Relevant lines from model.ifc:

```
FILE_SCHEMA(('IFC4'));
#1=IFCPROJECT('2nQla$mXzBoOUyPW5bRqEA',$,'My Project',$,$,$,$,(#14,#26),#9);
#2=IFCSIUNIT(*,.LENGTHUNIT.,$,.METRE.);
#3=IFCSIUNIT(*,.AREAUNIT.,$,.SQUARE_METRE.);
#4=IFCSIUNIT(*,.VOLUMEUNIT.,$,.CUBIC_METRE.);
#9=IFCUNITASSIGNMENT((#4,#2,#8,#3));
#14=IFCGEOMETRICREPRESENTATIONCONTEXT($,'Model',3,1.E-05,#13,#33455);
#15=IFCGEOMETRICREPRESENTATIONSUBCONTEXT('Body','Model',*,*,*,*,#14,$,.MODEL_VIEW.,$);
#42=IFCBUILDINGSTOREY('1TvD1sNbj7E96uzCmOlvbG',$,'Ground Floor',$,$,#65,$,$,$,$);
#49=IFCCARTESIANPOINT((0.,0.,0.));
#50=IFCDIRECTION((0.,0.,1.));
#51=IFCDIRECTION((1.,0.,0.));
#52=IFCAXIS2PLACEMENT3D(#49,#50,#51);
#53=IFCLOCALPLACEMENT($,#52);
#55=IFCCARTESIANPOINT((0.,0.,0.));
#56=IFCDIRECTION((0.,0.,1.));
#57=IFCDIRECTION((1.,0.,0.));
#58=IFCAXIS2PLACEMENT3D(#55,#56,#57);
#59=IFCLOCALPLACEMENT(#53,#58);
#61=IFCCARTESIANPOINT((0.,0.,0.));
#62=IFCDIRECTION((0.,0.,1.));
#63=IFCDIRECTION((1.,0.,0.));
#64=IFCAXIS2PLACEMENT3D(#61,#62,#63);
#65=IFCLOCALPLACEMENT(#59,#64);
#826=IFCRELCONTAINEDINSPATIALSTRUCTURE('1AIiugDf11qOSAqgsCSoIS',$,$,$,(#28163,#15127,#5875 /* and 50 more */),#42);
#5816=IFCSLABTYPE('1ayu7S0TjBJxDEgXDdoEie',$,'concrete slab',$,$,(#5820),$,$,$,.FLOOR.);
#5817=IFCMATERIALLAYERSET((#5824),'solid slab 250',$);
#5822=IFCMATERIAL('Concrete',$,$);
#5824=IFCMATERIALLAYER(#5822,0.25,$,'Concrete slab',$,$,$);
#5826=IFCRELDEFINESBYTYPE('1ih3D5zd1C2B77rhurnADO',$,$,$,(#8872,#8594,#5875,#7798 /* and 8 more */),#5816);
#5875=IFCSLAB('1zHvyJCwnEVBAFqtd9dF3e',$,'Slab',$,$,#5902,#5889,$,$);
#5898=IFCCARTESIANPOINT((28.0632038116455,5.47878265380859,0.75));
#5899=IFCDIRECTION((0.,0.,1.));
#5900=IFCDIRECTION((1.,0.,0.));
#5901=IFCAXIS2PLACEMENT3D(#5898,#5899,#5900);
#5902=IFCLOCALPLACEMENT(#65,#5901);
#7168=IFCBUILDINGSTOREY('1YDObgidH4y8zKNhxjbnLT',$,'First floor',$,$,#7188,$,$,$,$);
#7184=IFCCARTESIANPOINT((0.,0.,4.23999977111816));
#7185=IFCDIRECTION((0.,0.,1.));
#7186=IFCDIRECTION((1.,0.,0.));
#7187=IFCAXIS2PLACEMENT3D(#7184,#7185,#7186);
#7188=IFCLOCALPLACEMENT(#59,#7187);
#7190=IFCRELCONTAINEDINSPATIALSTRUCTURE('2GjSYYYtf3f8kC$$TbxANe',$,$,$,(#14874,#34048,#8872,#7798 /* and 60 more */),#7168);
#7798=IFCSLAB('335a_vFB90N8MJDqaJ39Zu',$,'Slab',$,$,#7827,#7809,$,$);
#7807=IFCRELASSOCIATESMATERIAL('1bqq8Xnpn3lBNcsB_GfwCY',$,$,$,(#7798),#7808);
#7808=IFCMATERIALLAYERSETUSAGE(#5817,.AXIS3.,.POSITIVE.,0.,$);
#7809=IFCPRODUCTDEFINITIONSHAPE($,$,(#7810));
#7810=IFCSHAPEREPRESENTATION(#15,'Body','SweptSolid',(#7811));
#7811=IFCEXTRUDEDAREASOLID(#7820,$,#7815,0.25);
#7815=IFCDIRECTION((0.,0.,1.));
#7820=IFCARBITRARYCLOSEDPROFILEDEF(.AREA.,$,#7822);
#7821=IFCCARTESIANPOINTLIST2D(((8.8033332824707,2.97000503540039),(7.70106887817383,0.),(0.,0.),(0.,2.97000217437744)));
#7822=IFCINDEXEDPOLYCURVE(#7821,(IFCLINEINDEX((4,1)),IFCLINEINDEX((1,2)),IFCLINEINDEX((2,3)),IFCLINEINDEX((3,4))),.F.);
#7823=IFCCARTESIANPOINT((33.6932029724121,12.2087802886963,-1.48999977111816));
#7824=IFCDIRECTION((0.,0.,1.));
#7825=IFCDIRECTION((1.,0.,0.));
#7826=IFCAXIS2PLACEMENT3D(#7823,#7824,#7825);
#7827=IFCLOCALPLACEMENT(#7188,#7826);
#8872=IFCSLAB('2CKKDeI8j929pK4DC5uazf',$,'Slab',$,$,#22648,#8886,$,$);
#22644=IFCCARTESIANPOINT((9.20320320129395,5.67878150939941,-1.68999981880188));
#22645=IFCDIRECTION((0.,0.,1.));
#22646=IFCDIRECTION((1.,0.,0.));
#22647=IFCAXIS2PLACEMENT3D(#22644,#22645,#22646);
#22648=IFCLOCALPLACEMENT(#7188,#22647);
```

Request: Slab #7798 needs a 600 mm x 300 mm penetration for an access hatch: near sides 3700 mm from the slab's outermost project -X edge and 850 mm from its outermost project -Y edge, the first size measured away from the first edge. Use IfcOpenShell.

```python
import numpy as np
import ifcopenshell
import ifcopenshell.api.feature
import ifcopenshell.api.geometry
import ifcopenshell.api.root
import ifcopenshell.geom
import ifcopenshell.util.placement
import ifcopenshell.util.representation
import ifcopenshell.util.shape
import ifcopenshell.util.unit

model = ifcopenshell.open("model.ifc")
unit_scale = ifcopenshell.util.unit.calculate_unit_scale(model)
settings = ifcopenshell.geom.settings()


def volume(element):
    """Net volume in cubic metres, openings subtracted."""
    shape = ifcopenshell.geom.create_shape(settings, element)
    return ifcopenshell.util.shape.get_volume(shape.geometry)


slab = model.by_guid("335a_vFB90N8MJDqaJ39Zu")
before = volume(slab)

# Extent in the slab's own axes, in metres. The edges named are its -X and -Y sides.
slab_shape = ifcopenshell.geom.create_shape(settings, slab)
vertices = ifcopenshell.util.shape.get_vertices(slab_shape.geometry)
x_min, y_min, bottom = vertices.min(axis=0)
top = vertices[:, 2].max()

opening = ifcopenshell.api.root.create_entity(model, ifc_class="IfcOpeningElement", name="Access hatch opening", predefined_type="OPENING")
context = ifcopenshell.util.representation.get_context(model, "Model", "Body", "MODEL_VIEW")
width, depth = 0.6, 0.3
outline = [(0.0, 0.0), (width, 0.0), (width, depth), (0.0, depth), (0.0, 0.0)]
# Overshoot both faces by 50 mm so the cut is clean.
shape = ifcopenshell.api.geometry.add_slab_representation(
    model, context=context, depth=top - bottom + 0.1, polyline=outline
)
ifcopenshell.api.geometry.assign_representation(model, product=opening, representation=shape)

matrix = ifcopenshell.util.placement.get_local_placement(slab.ObjectPlacement)
matrix[:, 3] = matrix @ np.append(np.array([x_min + 3.7, y_min + 0.85, bottom - 0.05]) / unit_scale, 1.0)
ifcopenshell.api.geometry.edit_object_placement(model, product=opening, matrix=matrix, is_si=False)
ifcopenshell.api.feature.add_feature(model, feature=opening, element=slab)

after = volume(slab)

print(f"slab volume {before:.3f} -> {after:.3f} m3")

model.write("model_v2.ifc")
```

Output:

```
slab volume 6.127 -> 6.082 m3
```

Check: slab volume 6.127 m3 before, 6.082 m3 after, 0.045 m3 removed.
